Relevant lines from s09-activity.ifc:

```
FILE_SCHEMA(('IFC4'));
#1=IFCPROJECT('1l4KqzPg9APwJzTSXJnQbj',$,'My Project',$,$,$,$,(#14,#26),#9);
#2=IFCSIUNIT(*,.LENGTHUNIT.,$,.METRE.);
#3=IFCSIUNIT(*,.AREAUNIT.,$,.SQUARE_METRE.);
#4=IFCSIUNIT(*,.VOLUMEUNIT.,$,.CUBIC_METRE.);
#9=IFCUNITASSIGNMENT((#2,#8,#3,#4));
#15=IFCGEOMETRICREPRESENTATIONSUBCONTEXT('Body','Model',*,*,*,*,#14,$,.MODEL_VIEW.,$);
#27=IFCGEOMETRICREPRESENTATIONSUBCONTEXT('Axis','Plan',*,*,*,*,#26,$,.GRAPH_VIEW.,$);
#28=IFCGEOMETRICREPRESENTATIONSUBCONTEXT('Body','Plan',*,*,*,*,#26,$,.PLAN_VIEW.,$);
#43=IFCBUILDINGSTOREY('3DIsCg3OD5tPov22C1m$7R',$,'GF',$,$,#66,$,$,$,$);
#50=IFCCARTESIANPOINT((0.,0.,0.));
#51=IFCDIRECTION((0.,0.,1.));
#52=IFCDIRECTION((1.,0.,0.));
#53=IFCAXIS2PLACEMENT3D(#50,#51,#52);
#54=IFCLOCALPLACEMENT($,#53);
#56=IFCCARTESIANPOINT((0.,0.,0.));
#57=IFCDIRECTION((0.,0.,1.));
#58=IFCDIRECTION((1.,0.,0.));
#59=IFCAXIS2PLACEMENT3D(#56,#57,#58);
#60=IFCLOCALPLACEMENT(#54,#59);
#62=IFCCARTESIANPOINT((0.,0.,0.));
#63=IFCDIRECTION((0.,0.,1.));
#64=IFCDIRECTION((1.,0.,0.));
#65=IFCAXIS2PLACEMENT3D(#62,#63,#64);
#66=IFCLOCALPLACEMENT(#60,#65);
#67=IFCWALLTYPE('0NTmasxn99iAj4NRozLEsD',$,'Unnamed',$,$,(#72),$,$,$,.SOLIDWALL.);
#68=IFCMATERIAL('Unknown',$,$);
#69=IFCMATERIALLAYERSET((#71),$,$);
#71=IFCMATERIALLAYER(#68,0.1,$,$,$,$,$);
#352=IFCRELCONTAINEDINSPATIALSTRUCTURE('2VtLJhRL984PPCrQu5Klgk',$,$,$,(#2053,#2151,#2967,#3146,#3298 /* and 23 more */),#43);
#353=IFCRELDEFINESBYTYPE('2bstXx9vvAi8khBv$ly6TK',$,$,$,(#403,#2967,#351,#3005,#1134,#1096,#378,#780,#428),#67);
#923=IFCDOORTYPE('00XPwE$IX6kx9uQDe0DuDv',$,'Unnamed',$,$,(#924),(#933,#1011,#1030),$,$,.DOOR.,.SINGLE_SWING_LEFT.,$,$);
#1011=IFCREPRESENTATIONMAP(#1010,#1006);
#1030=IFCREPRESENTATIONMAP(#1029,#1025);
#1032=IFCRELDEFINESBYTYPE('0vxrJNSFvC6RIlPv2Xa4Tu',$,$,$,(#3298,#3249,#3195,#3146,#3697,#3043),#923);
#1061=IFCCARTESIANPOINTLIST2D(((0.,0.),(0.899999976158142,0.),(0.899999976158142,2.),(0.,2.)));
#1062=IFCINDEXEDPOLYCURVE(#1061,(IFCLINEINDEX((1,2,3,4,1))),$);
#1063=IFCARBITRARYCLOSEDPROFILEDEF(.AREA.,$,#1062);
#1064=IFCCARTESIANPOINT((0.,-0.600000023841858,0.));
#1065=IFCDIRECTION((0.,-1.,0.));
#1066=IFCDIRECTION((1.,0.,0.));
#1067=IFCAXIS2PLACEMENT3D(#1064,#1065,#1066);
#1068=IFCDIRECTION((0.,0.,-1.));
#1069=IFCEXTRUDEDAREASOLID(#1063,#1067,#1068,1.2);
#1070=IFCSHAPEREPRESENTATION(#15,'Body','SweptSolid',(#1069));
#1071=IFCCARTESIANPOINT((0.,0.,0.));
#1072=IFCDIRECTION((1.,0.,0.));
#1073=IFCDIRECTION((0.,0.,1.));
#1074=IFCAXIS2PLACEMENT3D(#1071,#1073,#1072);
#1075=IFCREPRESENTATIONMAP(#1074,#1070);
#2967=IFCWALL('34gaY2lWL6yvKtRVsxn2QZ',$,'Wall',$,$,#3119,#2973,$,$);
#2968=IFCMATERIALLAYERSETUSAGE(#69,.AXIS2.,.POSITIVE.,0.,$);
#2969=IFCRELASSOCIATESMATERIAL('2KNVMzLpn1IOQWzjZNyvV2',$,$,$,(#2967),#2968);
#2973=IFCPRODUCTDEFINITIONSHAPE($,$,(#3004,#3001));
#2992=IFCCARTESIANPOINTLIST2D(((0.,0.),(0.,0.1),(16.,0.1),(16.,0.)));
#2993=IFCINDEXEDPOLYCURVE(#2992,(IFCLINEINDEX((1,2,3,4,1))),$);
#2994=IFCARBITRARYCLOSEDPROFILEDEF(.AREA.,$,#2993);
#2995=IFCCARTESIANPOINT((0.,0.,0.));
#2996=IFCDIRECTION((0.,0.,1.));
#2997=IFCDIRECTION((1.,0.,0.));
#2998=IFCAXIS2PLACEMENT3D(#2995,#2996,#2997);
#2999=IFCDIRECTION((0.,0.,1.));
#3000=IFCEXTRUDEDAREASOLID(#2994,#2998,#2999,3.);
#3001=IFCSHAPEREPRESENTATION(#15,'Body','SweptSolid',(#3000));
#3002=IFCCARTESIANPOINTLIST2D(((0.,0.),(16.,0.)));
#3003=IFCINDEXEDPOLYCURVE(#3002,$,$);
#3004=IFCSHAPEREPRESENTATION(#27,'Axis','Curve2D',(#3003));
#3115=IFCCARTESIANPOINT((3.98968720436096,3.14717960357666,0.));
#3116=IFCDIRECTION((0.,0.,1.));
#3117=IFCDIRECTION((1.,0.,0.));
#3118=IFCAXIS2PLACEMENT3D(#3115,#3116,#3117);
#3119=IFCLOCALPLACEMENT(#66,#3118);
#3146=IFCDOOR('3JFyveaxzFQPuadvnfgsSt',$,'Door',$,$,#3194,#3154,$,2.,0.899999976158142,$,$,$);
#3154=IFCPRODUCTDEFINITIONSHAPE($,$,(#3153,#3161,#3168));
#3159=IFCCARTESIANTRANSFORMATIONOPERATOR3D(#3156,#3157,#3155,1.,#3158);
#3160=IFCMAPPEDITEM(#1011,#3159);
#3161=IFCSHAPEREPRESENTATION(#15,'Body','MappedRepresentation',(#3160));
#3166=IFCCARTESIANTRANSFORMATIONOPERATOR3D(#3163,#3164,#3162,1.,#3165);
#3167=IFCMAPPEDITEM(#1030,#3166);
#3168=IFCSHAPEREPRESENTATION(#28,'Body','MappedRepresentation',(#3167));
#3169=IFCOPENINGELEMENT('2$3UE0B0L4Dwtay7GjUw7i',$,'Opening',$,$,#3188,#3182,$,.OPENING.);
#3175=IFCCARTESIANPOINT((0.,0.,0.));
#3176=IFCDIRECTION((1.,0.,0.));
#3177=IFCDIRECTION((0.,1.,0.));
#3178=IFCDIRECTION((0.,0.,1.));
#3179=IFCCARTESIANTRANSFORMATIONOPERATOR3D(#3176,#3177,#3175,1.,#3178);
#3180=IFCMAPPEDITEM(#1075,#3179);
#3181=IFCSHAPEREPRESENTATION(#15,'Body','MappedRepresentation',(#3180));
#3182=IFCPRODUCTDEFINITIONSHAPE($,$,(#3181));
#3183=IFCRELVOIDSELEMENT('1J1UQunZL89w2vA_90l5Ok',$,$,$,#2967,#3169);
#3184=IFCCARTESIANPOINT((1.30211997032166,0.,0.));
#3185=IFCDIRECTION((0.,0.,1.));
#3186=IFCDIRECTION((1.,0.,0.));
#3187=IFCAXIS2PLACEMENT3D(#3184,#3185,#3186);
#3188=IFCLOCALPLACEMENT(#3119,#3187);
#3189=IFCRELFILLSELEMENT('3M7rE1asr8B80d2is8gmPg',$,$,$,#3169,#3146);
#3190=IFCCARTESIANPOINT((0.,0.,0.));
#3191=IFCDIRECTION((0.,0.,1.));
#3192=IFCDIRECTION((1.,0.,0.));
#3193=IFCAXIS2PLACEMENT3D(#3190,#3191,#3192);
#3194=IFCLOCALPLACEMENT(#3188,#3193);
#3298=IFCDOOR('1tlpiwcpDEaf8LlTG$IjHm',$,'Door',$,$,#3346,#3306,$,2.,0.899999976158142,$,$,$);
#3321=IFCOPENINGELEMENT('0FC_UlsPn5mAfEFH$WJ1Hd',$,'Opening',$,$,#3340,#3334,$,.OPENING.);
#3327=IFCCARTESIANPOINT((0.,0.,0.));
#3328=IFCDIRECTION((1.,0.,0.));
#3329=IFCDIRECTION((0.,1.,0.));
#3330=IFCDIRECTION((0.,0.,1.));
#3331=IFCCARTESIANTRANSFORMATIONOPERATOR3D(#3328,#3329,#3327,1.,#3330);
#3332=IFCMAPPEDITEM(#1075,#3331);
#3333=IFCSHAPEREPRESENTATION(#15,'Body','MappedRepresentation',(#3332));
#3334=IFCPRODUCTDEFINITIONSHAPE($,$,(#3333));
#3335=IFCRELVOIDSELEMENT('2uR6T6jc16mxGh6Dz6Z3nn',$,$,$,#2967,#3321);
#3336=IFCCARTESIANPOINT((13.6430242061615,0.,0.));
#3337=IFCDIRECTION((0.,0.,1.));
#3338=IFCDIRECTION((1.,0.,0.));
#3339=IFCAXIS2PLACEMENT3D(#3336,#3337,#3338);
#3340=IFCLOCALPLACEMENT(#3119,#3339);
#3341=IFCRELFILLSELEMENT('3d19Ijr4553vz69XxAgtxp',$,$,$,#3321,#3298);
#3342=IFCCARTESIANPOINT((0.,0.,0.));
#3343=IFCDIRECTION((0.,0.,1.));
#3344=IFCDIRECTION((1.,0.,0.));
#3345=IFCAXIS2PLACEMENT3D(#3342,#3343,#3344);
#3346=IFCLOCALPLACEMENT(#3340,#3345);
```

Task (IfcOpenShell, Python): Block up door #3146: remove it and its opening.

```python
import ifcopenshell
import ifcopenshell.api.feature
import ifcopenshell.api.root
import ifcopenshell.geom
import ifcopenshell.util.shape

model = ifcopenshell.open("s09-activity.ifc")
settings = ifcopenshell.geom.settings()


def volume(element):
    """Net volume in cubic metres, openings subtracted."""
    shape = ifcopenshell.geom.create_shape(settings, element)
    return ifcopenshell.util.shape.get_volume(shape.geometry)


door = model.by_guid("3JFyveaxzFQPuadvnfgsSt")
opening = door.FillsVoids[0].RelatingOpeningElement
wall = opening.VoidsElements[0].RelatingBuildingElement
before = volume(wall)

ifcopenshell.api.root.remove_product(model, product=door)
ifcopenshell.api.feature.remove_feature(model, feature=opening)

after = volume(wall)

print(f"wall volume {before:.3f} -> {after:.3f} m3")

model.write("s09-activity_rev.ifc")
```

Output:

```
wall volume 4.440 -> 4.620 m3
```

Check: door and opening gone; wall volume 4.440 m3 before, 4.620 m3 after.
